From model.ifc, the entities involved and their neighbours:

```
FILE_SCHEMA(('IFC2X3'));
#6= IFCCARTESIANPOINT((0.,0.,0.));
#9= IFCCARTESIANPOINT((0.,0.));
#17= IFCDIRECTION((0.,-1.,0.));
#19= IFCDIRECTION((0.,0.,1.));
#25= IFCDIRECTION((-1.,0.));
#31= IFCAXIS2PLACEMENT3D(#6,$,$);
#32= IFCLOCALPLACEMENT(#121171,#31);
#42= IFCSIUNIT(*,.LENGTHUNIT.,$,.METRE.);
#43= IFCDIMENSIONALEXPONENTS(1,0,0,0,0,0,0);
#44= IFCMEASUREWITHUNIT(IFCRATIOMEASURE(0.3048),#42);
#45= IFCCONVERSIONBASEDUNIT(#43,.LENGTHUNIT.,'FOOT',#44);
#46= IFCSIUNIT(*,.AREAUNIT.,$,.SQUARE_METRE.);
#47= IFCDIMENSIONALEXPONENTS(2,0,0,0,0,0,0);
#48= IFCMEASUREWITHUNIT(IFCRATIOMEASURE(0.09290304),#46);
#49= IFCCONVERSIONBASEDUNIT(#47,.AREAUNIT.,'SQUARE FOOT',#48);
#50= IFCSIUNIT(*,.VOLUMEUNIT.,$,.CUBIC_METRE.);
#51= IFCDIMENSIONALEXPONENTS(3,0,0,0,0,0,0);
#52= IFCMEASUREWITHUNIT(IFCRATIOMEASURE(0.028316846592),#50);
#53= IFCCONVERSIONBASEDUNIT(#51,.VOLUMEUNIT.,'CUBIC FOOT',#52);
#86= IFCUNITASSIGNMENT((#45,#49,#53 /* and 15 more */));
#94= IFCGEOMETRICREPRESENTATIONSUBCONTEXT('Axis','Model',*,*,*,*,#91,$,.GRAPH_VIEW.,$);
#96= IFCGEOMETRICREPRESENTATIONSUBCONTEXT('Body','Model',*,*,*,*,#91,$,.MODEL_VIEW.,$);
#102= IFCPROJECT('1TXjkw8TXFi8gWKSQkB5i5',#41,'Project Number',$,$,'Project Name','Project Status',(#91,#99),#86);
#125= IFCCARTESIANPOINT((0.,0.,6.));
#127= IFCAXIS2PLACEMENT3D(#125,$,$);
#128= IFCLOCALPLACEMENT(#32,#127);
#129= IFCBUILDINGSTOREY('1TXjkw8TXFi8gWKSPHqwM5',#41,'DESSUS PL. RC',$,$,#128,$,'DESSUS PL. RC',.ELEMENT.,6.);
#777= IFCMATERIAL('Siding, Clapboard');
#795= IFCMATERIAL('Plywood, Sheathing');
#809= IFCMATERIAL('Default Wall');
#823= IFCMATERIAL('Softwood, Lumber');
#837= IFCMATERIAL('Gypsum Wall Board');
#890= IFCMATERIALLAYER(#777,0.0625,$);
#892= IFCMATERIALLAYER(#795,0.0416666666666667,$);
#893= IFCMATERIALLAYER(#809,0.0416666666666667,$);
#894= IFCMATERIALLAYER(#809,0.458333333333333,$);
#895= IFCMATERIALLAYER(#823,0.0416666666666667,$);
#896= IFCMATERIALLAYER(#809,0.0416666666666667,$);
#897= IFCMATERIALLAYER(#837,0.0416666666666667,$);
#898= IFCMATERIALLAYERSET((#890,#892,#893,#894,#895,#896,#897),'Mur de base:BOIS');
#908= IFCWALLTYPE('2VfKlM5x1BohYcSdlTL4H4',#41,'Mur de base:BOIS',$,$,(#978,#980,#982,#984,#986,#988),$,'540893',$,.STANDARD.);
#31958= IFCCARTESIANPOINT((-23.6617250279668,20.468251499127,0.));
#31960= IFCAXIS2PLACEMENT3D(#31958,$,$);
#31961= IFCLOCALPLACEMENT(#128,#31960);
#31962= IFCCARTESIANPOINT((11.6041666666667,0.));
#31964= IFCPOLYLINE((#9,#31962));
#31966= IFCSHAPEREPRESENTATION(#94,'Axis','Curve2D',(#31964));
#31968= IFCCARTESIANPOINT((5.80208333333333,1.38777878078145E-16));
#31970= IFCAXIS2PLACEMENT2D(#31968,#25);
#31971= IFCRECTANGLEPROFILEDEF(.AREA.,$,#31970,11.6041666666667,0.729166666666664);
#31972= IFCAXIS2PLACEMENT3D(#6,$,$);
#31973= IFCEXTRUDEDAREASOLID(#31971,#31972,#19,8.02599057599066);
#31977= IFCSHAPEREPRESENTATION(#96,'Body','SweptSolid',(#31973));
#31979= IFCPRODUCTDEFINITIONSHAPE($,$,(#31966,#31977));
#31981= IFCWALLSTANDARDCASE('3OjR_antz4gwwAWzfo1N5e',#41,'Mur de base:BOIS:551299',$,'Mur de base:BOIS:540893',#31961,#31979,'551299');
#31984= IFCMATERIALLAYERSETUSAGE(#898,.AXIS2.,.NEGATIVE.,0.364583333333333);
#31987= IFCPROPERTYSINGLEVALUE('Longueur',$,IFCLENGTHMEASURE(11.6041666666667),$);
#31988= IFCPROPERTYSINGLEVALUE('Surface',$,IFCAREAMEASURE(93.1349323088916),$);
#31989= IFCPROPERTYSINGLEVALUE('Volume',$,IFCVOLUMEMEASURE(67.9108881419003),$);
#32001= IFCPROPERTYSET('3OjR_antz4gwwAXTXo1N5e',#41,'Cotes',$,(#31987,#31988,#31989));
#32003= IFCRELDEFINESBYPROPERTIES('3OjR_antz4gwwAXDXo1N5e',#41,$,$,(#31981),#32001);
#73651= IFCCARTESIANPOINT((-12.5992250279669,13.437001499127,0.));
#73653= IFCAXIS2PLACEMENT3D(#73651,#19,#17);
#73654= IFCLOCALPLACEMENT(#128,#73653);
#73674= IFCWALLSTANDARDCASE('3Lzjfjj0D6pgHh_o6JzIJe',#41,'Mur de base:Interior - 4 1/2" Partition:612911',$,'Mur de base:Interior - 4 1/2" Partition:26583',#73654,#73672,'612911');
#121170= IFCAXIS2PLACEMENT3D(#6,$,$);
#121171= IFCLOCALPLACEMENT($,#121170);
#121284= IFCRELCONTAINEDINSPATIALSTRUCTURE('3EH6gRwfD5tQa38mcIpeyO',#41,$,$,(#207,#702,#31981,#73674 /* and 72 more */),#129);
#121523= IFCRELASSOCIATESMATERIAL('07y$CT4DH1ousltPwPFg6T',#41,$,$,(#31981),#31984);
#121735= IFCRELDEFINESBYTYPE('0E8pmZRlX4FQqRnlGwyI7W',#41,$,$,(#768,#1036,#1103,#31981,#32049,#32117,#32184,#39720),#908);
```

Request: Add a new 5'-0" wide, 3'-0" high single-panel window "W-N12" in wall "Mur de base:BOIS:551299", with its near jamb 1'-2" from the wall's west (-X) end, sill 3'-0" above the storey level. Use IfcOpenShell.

```python
import numpy as np
import ifcopenshell
import ifcopenshell.api.feature
import ifcopenshell.api.geometry
import ifcopenshell.api.pset
import ifcopenshell.api.root
import ifcopenshell.api.spatial
import ifcopenshell.api.type
import ifcopenshell.geom
import ifcopenshell.util.element
import ifcopenshell.util.placement
import ifcopenshell.util.representation
import ifcopenshell.util.shape
import ifcopenshell.util.unit

model = ifcopenshell.open("model.ifc")
unit_scale = ifcopenshell.util.unit.calculate_unit_scale(model)
area_scale = ifcopenshell.util.unit.calculate_unit_scale(model, "AREAUNIT")
volume_scale = ifcopenshell.util.unit.calculate_unit_scale(model, "VOLUMEUNIT")
settings = ifcopenshell.geom.settings()


def volume(element):
    """Net volume in cubic metres, openings subtracted."""
    shape = ifcopenshell.geom.create_shape(settings, element)
    return ifcopenshell.util.shape.get_volume(shape.geometry)


wall = model.by_guid("3OjR_antz4gwwAWzfo1N5e")
storey = ifcopenshell.util.element.get_container(wall, ifc_class="IfcBuildingStorey")
context = ifcopenshell.util.representation.get_context(model, "Model", "Body", "MODEL_VIEW")
before = volume(wall)

width, height, from_end, sill = 1.524, 0.9144, 0.3556, 0.9144  # metres

# The wall runs along its own X axis, and the end named is its -X end.
wall_shape = ifcopenshell.geom.create_shape(settings, wall)
x, y, z = ifcopenshell.util.shape.get_vertices(wall_shape.geometry).T
start = x.min() + from_end
face, thickness = float(y.min()), float(y.max() - y.min())
wall_matrix = ifcopenshell.util.placement.get_local_placement(wall.ObjectPlacement)
level = ifcopenshell.util.placement.get_local_placement(storey.ObjectPlacement)[2, 3]


def in_wall(x, y):
    """Placement at x, y metres in the wall's axes, at sill height."""
    matrix = wall_matrix.copy()
    matrix[:, 3] = wall_matrix @ np.array([x / unit_scale, y / unit_scale, 0.0, 1.0])
    matrix[2, 3] = level + sill / unit_scale
    return matrix


# Opening: a box that overshoots both wall faces by 50 mm.
opening = ifcopenshell.api.root.create_entity(model, ifc_class="IfcOpeningElement")
box = ifcopenshell.api.geometry.add_wall_representation(
    model, context=context, length=width, height=height, thickness=thickness + 0.1
)
ifcopenshell.api.geometry.assign_representation(model, product=opening, representation=box)
ifcopenshell.api.geometry.edit_object_placement(model, product=opening, matrix=in_wall(start, face - 0.05), is_si=False)
ifcopenshell.api.feature.add_feature(model, feature=opening, element=wall)

window = ifcopenshell.api.root.create_entity(model, ifc_class="IfcWindow", name="W-N12")
window.OverallWidth, window.OverallHeight = width / unit_scale, height / unit_scale
body = ifcopenshell.api.geometry.add_window_representation(
    model,
    context=context,
    overall_width=window.OverallWidth,
    overall_height=window.OverallHeight,
    partition_type="SINGLE_PANEL",
)
ifcopenshell.api.geometry.assign_representation(model, product=window, representation=body)
ifcopenshell.api.spatial.assign_container(model, products=[window], relating_structure=storey)
fills = ifcopenshell.api.feature.add_filling(model, opening=opening, element=window)
fills.OwnerHistory = window.OwnerHistory  # required in IFC2X3

# IFC2X3 keeps the operation on the window style.
style = ifcopenshell.api.root.create_entity(model, ifc_class="IfcWindowStyle", name="W-N12")
style.OperationType, style.ConstructionType = "SINGLE_PANEL", "NOTDEFINED"
style.ParameterTakesPrecedence = style.Sizeable = False
ifcopenshell.api.type.assign_type(model, related_objects=[window], relating_type=style)

# Centre the window in the wall's thickness.
ifcopenshell.api.geometry.edit_object_placement(model, product=window, matrix=in_wall(start, face), is_si=False)
window_shape = ifcopenshell.geom.create_shape(settings, window)
depth = ifcopenshell.util.shape.get_vertices(window_shape.geometry)[:, 1]
offset = face + thickness / 2 - (depth.min() + depth.max()) / 2
ifcopenshell.api.geometry.edit_object_placement(model, product=window, matrix=in_wall(start, offset), is_si=False)

after = volume(wall)

# Update the wall's stored quantities.
pset = model.by_id(ifcopenshell.util.element.get_pset(wall, "Cotes", should_inherit=False)["id"])
ifcopenshell.api.pset.edit_pset(model, pset=pset, properties={
    "Surface": model.create_entity("IfcAreaMeasure", after / thickness / area_scale),
    "Volume": model.create_entity("IfcVolumeMeasure", after / volume_scale),
})

print(f"wall volume {before:.3f} -> {after:.3f} m3")

model.write("model_updated.ifc")
```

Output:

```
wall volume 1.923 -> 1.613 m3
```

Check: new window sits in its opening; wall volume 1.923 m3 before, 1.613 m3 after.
